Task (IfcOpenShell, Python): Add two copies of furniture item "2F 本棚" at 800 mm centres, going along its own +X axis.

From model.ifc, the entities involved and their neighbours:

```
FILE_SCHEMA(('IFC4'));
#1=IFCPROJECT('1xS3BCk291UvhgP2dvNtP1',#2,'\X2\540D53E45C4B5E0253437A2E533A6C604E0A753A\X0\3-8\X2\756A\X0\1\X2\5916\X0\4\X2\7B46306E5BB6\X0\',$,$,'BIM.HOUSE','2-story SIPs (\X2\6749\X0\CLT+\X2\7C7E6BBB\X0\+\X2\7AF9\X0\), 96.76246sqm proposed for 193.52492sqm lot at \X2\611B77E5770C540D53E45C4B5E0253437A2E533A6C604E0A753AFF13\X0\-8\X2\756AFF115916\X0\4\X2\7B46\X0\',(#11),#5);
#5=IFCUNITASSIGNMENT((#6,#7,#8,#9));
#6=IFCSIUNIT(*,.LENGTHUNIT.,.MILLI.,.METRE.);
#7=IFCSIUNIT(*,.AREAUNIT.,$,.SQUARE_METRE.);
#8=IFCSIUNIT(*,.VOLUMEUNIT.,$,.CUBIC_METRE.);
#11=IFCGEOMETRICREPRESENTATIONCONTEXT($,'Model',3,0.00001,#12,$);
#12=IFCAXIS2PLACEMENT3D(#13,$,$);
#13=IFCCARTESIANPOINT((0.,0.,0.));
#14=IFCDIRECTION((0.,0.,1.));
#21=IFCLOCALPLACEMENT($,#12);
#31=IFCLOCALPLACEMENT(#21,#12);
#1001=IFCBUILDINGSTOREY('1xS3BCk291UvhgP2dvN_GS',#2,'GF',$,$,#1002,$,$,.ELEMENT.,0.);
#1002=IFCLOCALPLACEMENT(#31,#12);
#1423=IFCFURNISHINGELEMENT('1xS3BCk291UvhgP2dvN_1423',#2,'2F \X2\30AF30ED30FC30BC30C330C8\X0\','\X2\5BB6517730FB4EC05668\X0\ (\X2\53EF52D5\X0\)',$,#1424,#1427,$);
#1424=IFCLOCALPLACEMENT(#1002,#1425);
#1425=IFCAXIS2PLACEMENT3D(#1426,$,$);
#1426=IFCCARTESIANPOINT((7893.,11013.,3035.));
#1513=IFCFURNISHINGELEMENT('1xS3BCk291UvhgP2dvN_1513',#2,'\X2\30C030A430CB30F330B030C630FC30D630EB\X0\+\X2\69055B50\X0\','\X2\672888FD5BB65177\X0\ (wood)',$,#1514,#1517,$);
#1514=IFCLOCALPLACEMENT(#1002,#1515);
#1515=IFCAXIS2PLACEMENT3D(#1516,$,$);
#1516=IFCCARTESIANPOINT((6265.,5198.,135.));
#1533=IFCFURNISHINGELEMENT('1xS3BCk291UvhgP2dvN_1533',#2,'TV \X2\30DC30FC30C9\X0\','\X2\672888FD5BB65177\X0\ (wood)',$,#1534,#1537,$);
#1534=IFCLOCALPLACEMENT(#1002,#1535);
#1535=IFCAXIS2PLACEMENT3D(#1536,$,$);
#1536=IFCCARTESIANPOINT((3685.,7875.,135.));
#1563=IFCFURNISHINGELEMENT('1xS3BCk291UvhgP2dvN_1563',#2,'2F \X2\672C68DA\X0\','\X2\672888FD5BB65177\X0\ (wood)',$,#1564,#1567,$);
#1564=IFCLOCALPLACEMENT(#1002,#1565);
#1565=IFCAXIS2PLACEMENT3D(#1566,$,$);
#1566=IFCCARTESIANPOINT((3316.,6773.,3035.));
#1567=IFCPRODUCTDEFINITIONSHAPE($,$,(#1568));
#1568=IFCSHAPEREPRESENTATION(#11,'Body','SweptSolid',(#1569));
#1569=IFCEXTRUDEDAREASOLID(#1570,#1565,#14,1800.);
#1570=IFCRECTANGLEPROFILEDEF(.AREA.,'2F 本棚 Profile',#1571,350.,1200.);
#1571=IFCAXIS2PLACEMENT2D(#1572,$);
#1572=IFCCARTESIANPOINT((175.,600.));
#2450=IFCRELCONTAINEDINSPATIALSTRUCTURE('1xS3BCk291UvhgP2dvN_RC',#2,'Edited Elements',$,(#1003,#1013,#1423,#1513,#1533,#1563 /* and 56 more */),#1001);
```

```python
import ifcopenshell
import ifcopenshell.api.geometry
import ifcopenshell.api.root
import ifcopenshell.util.element
import ifcopenshell.util.placement

model = ifcopenshell.open("model.ifc")


def reuse_history(source, copy):
    """copy_class also copies each property set's owner history, people and application; keep the originals."""
    for rel in copy.IsDefinedBy:
        if rel.is_a("IfcRelDefinesByProperties") and (history := rel.RelatingPropertyDefinition.OwnerHistory):
            rel.RelatingPropertyDefinition.OwnerHistory = source.OwnerHistory
            ifcopenshell.util.element.remove_deep2(model, history)


source = model.by_guid("1xS3BCk291UvhgP2dvN_1563")
base = ifcopenshell.util.placement.get_local_placement(source.ObjectPlacement)
step = base[:3, 0] * 800.0

for i in range(1, 3):
    copy = ifcopenshell.api.root.copy_class(model, product=source)
    copy.Representation = ifcopenshell.util.element.copy_deep(
        model, source.Representation, exclude=["IfcGeometricRepresentationContext", "IfcRepresentationMap"]
    )
    reuse_history(source, copy)
    matrix = base.copy()
    matrix[:3, 3] += i * step
    print("added at", matrix[:3, 3].round(3) + 0.0)
    ifcopenshell.api.geometry.edit_object_placement(model, product=copy, matrix=matrix, is_si=False)

model.write("model_rev.ifc")
```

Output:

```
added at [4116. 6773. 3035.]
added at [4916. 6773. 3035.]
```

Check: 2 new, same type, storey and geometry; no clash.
